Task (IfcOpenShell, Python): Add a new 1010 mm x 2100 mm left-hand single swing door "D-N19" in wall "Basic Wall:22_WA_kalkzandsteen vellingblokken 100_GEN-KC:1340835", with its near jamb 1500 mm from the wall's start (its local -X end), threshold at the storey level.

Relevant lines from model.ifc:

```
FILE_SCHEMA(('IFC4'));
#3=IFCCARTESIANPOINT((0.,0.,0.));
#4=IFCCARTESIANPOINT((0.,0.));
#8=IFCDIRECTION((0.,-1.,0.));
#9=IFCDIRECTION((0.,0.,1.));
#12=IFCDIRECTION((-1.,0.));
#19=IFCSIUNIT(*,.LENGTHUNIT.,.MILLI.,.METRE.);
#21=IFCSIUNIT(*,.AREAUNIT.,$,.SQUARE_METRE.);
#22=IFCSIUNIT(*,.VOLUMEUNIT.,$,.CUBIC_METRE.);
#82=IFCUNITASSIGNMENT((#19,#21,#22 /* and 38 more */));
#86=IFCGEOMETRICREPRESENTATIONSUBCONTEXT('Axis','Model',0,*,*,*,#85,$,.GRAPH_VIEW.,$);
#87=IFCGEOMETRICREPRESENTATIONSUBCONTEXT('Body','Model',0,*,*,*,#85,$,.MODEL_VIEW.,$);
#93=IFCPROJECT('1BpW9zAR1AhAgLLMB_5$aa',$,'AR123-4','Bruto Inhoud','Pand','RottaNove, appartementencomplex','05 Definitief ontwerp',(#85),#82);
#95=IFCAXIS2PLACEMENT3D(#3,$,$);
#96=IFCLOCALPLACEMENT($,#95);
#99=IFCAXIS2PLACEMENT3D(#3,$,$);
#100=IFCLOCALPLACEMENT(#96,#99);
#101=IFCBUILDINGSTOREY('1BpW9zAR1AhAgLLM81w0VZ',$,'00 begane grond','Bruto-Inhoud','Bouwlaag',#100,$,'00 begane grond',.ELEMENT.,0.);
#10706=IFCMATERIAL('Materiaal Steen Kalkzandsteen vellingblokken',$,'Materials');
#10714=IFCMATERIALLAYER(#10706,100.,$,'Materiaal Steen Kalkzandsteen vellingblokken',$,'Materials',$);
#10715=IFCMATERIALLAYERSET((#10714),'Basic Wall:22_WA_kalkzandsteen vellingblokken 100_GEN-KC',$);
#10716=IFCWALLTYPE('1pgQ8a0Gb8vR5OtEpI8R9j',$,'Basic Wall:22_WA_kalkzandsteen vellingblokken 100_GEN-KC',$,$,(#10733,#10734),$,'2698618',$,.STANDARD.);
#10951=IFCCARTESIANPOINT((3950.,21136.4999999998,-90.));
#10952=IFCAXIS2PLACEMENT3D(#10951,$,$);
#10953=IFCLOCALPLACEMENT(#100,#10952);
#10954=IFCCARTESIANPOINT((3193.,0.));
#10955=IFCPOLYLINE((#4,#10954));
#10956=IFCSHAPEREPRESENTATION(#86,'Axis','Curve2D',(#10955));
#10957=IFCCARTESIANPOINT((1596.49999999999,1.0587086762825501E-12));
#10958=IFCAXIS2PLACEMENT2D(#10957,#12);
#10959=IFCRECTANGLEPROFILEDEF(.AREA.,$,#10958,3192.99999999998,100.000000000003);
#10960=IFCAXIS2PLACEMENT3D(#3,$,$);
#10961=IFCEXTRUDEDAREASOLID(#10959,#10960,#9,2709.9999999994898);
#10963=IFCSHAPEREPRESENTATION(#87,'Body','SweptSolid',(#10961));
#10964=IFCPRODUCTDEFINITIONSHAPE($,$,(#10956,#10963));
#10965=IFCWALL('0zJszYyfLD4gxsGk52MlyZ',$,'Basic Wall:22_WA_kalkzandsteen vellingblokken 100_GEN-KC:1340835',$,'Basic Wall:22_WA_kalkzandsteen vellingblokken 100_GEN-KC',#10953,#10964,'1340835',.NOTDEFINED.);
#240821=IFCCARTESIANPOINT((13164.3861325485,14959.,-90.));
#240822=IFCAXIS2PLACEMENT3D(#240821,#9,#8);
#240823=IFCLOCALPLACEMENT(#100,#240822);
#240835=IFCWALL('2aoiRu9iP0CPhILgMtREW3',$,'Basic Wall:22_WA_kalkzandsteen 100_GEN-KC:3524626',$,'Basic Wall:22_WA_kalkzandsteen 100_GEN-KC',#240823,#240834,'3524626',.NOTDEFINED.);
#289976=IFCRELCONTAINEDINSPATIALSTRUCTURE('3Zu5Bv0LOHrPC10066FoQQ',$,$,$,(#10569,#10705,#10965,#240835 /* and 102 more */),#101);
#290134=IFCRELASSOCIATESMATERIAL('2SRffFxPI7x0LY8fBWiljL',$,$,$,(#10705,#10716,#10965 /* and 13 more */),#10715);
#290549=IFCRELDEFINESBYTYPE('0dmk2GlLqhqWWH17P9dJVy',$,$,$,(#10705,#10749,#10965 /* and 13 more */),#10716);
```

```python
import numpy as np
import ifcopenshell
import ifcopenshell.api.feature
import ifcopenshell.api.geometry
import ifcopenshell.api.root
import ifcopenshell.api.spatial
import ifcopenshell.geom
import ifcopenshell.util.element
import ifcopenshell.util.placement
import ifcopenshell.util.representation
import ifcopenshell.util.shape
import ifcopenshell.util.unit

model = ifcopenshell.open("model.ifc")
unit_scale = ifcopenshell.util.unit.calculate_unit_scale(model)
settings = ifcopenshell.geom.settings()


def volume(element):
    """Net volume in cubic metres, openings subtracted."""
    shape = ifcopenshell.geom.create_shape(settings, element)
    return ifcopenshell.util.shape.get_volume(shape.geometry)


wall = model.by_guid("0zJszYyfLD4gxsGk52MlyZ")
storey = ifcopenshell.util.element.get_container(wall, ifc_class="IfcBuildingStorey")
context = ifcopenshell.util.representation.get_context(model, "Model", "Body", "MODEL_VIEW")
before = volume(wall)

width, height, from_end, sill = 1.01, 2.1, 1.5, 0.0  # metres

# The wall runs along its own X axis, and the end named is its -X end.
wall_shape = ifcopenshell.geom.create_shape(settings, wall)
x, y, z = ifcopenshell.util.shape.get_vertices(wall_shape.geometry).T
start = x.min() + from_end
face, thickness = float(y.min()), float(y.max() - y.min())
wall_matrix = ifcopenshell.util.placement.get_local_placement(wall.ObjectPlacement)
level = ifcopenshell.util.placement.get_local_placement(storey.ObjectPlacement)[2, 3]


def in_wall(x, y):
    """Placement at x, y metres in the wall's axes, at sill height."""
    matrix = wall_matrix.copy()
    matrix[:, 3] = wall_matrix @ np.array([x / unit_scale, y / unit_scale, 0.0, 1.0])
    matrix[2, 3] = level + sill / unit_scale
    return matrix


# Opening: a box that overshoots both wall faces by 50 mm.
opening = ifcopenshell.api.root.create_entity(model, ifc_class="IfcOpeningElement", predefined_type="OPENING")
box = ifcopenshell.api.geometry.add_wall_representation(
    model, context=context, length=width, height=height, thickness=thickness + 0.1
)
ifcopenshell.api.geometry.assign_representation(model, product=opening, representation=box)
ifcopenshell.api.geometry.edit_object_placement(model, product=opening, matrix=in_wall(start, face - 0.05), is_si=False)
ifcopenshell.api.feature.add_feature(model, feature=opening, element=wall)

door = ifcopenshell.api.root.create_entity(model, ifc_class="IfcDoor", name="D-N19", predefined_type="DOOR")
door.OverallWidth, door.OverallHeight = width / unit_scale, height / unit_scale
door.OperationType = "SINGLE_SWING_LEFT"
body = ifcopenshell.api.geometry.add_door_representation(
    model,
    context=context,
    overall_width=door.OverallWidth,
    overall_height=door.OverallHeight,
    operation_type="SINGLE_SWING_LEFT",
    lining_properties={"LiningDepth": thickness / unit_scale, "ThresholdDepth": thickness / unit_scale},
)
ifcopenshell.api.geometry.assign_representation(model, product=door, representation=body)
ifcopenshell.api.spatial.assign_container(model, products=[door], relating_structure=storey)
ifcopenshell.api.feature.add_filling(model, opening=opening, element=door)

# The lining spans the wall, so the door starts at the wall face.
ifcopenshell.api.geometry.edit_object_placement(model, product=door, matrix=in_wall(start, face), is_si=False)

after = volume(wall)

print(f"wall volume {before:.3f} -> {after:.3f} m3")

model.write("model_updated.ifc")
```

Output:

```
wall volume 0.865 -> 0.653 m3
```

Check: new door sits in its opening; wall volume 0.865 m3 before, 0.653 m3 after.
